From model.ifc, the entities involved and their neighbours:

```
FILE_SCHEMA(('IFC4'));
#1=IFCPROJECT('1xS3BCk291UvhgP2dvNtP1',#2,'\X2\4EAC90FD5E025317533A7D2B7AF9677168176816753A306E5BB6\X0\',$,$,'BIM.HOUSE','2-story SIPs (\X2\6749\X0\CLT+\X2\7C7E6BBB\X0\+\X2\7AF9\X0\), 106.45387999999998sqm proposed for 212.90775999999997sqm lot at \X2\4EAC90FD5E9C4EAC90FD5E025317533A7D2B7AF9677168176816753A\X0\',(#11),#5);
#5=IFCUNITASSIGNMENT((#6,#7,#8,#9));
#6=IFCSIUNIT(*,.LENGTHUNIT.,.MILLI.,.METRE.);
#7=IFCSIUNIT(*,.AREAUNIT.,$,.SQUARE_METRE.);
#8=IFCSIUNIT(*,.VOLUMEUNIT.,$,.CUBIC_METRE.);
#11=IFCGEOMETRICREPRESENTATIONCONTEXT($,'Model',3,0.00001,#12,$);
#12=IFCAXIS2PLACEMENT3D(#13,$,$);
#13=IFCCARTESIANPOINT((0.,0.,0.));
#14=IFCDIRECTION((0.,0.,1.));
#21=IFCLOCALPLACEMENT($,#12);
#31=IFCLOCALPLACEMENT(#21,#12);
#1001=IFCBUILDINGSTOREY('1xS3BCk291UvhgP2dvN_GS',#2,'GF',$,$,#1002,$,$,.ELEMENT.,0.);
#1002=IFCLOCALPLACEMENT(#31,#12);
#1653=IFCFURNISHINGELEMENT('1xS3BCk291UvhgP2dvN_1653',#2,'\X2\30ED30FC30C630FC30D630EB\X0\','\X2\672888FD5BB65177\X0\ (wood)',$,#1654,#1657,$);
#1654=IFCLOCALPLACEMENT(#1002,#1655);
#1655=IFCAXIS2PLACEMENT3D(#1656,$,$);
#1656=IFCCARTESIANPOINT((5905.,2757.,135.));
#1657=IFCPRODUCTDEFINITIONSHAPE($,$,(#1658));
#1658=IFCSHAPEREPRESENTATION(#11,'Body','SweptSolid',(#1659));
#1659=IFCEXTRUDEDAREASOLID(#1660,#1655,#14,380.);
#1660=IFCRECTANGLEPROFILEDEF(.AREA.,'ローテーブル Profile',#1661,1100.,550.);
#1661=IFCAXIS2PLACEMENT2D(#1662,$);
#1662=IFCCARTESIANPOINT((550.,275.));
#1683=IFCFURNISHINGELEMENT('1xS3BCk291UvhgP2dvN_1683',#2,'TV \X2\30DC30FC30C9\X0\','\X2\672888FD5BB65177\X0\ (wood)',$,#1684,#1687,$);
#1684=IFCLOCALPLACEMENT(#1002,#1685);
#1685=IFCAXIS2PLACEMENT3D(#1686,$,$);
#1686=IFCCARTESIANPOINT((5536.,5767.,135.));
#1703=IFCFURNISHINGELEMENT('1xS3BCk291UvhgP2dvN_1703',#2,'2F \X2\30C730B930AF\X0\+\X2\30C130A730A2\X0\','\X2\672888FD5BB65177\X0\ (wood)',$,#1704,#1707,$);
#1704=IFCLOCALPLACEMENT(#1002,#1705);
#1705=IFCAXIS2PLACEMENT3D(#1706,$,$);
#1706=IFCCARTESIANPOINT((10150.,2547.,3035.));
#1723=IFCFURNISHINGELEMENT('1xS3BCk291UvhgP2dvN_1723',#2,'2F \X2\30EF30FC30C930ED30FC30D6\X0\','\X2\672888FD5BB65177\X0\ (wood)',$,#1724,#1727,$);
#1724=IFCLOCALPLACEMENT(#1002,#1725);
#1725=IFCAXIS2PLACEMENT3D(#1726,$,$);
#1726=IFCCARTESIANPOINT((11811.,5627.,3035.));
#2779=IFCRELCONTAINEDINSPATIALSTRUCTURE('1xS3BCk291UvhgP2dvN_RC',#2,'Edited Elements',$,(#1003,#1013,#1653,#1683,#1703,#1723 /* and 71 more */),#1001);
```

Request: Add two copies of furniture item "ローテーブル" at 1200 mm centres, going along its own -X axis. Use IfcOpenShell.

```python
import ifcopenshell
import ifcopenshell.api.geometry
import ifcopenshell.api.root
import ifcopenshell.util.element
import ifcopenshell.util.placement

model = ifcopenshell.open("model.ifc")


def reuse_history(source, copy):
    """copy_class also copies each property set's owner history, people and application; keep the originals."""
    for rel in copy.IsDefinedBy:
        if rel.is_a("IfcRelDefinesByProperties") and (history := rel.RelatingPropertyDefinition.OwnerHistory):
            rel.RelatingPropertyDefinition.OwnerHistory = source.OwnerHistory
            ifcopenshell.util.element.remove_deep2(model, history)


source = model.by_guid("1xS3BCk291UvhgP2dvN_1653")
base = ifcopenshell.util.placement.get_local_placement(source.ObjectPlacement)
step = -base[:3, 0] * 1200.0

for i in range(1, 3):
    copy = ifcopenshell.api.root.copy_class(model, product=source)
    copy.Representation = ifcopenshell.util.element.copy_deep(
        model, source.Representation, exclude=["IfcGeometricRepresentationContext", "IfcRepresentationMap"]
    )
    reuse_history(source, copy)
    matrix = base.copy()
    matrix[:3, 3] += i * step
    print("added at", matrix[:3, 3].round(3) + 0.0)
    ifcopenshell.api.geometry.edit_object_placement(model, product=copy, matrix=matrix, is_si=False)

model.write("model-out.ifc")
```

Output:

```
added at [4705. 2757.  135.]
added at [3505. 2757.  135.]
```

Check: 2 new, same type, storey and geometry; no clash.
